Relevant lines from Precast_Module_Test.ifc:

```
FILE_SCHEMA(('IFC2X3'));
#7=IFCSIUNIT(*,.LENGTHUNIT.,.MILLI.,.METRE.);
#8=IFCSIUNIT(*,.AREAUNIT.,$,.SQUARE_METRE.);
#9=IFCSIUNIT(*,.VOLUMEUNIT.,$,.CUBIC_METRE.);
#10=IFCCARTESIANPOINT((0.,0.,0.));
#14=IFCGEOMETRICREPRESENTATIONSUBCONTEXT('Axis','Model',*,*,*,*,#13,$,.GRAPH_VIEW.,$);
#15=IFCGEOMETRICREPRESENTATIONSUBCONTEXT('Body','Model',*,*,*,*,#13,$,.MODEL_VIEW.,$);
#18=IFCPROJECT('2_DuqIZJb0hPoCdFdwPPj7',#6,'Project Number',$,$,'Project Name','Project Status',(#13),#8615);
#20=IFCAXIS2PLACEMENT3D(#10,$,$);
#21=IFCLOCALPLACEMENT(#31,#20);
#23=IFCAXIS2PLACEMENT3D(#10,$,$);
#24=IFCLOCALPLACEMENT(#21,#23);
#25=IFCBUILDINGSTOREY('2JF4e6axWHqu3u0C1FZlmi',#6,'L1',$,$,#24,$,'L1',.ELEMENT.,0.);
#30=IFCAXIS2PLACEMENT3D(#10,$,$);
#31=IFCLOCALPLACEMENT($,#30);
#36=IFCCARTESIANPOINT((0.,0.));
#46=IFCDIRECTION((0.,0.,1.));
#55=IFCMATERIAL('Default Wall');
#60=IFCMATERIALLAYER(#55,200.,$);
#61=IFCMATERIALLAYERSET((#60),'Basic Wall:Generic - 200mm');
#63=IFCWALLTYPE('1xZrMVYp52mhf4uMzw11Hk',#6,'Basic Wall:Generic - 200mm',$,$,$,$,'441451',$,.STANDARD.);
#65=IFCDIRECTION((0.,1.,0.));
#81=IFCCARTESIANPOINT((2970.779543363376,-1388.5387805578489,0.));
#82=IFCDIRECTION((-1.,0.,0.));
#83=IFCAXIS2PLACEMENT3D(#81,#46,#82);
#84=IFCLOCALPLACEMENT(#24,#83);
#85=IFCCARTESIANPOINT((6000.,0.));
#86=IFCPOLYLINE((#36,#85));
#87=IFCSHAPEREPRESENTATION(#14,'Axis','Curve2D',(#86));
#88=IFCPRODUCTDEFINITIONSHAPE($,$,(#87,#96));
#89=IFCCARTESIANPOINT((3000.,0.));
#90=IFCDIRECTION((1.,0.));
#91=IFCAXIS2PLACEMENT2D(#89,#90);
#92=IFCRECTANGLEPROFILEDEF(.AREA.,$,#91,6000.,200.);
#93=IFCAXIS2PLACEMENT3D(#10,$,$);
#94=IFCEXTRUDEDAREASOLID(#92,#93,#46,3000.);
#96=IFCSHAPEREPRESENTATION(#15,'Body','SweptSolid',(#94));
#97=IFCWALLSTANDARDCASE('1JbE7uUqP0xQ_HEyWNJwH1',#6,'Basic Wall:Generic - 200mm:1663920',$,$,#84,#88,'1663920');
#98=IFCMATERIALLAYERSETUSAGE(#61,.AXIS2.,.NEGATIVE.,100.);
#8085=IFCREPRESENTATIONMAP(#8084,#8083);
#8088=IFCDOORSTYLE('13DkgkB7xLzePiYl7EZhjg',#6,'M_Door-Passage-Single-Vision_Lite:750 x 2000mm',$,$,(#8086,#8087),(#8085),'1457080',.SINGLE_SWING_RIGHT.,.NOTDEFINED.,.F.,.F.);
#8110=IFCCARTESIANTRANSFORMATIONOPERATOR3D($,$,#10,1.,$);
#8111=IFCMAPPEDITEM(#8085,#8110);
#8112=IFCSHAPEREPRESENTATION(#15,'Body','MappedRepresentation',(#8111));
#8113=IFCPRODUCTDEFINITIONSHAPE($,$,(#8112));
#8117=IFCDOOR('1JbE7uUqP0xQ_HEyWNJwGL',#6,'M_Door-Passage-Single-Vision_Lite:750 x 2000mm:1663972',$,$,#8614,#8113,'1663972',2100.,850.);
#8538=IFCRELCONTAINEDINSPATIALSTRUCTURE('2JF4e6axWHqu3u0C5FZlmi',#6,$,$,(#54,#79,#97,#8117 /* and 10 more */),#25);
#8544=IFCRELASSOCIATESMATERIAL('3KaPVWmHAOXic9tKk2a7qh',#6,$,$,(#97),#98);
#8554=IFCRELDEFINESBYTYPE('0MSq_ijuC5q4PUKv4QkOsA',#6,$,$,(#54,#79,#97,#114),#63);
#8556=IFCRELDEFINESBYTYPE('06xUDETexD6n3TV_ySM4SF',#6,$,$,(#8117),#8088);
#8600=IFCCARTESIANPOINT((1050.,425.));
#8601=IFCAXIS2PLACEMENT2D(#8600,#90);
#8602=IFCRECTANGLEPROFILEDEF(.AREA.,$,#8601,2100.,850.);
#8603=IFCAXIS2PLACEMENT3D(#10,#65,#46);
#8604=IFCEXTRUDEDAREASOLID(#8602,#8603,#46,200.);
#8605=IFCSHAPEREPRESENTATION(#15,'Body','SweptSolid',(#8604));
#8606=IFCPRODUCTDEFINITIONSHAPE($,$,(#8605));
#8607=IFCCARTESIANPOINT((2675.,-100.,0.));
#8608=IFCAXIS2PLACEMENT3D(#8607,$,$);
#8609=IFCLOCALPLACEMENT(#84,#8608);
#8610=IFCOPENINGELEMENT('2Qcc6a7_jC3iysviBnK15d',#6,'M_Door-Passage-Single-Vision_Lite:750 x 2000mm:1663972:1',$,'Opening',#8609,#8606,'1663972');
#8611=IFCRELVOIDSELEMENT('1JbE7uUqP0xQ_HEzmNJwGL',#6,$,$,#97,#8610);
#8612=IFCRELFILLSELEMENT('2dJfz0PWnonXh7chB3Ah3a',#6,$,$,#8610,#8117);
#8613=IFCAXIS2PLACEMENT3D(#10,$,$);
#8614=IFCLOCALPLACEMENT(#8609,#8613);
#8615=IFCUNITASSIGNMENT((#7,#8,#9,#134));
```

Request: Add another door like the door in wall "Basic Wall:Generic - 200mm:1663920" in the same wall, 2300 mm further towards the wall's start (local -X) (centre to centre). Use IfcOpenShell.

```python
import ifcopenshell
import ifcopenshell.api.feature
import ifcopenshell.api.geometry
import ifcopenshell.api.root
import ifcopenshell.geom
import ifcopenshell.util.element
import ifcopenshell.util.placement
import ifcopenshell.util.shape

model = ifcopenshell.open("Precast_Module_Test.ifc")
settings = ifcopenshell.geom.settings()


def volume(element):
    """Net volume in cubic metres, openings subtracted."""
    shape = ifcopenshell.geom.create_shape(settings, element)
    return ifcopenshell.util.shape.get_volume(shape.geometry)


door = model.by_id(8117)
opening = door.FillsVoids[0].RelatingOpeningElement
wall = opening.VoidsElements[0].RelatingBuildingElement
before = volume(wall)
shift = ifcopenshell.util.placement.get_local_placement(wall.ObjectPlacement)[:3, 0] * -2300.0

# copy_class copies the void relationship, type, container and properties, but no geometry.
new_opening = ifcopenshell.api.root.copy_class(model, product=opening)
new_opening.Representation = ifcopenshell.util.element.copy_deep(
    model, opening.Representation, exclude=["IfcGeometricRepresentationContext", "IfcRepresentationMap"]
)
new_opening.Name = "M_Door-Passage-Single-Vision_Lite:750 x 2000mm"
new_opening.Tag = None
new_door = ifcopenshell.api.root.copy_class(model, product=door)
new_door.Representation = ifcopenshell.util.element.copy_deep(
    model, door.Representation, exclude=["IfcGeometricRepresentationContext", "IfcRepresentationMap"]
)
new_door.Name = "M_Door-Passage-Single-Vision_Lite:750 x 2000mm"
new_door.Tag = None
fills = ifcopenshell.api.feature.add_filling(model, opening=new_opening, element=new_door)
fills.OwnerHistory = new_door.OwnerHistory  # required in IFC2X3

for old, new in ((opening, new_opening), (door, new_door)):
    matrix = ifcopenshell.util.placement.get_local_placement(old.ObjectPlacement)
    matrix[:3, 3] += shift
    ifcopenshell.api.geometry.edit_object_placement(model, product=new, matrix=matrix, is_si=False)

after = volume(wall)

print(f"wall volume {before:.3f} -> {after:.3f} m3")

model.write("Precast_Module_Test_updated.ifc")
```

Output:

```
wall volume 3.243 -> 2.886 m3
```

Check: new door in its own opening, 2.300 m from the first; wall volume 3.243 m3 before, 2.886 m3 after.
